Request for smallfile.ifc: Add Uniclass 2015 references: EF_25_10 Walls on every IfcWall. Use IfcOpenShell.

First a look at what the model holds.

```python
import ifcopenshell

model = ifcopenshell.open("smallfile.ifc")
print(model.schema)
print("classifications:", [c.Name for c in model.by_type("IfcClassification")])
for ifc_class in ("IfcDoor", "IfcRoof", "IfcStair", "IfcWall", "IfcWindow"):
    print(ifc_class, len(model.by_type(ifc_class)))
```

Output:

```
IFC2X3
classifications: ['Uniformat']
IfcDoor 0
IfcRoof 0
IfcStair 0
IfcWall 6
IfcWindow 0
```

```python
import ifcopenshell
import ifcopenshell.api.classification

model = ifcopenshell.open("smallfile.ifc")

# IFC2X3 requires Source and Edition and has no link from the project to the system.
system = model.create_entity("IfcClassification", Source="NBS", Edition="2015", Name="Uniclass 2015")

codes = {
    "IfcWall": ("EF_25_10", "Walls"),
}
for ifc_class, (code, name) in codes.items():
    products = model.by_type(ifc_class)
    ifcopenshell.api.classification.add_reference(
        model, products=products, classification=system, identification=code, name=name
    )
    print(code, len(products))

model.write("smallfile_updated.ifc")
```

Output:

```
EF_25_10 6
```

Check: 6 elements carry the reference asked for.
